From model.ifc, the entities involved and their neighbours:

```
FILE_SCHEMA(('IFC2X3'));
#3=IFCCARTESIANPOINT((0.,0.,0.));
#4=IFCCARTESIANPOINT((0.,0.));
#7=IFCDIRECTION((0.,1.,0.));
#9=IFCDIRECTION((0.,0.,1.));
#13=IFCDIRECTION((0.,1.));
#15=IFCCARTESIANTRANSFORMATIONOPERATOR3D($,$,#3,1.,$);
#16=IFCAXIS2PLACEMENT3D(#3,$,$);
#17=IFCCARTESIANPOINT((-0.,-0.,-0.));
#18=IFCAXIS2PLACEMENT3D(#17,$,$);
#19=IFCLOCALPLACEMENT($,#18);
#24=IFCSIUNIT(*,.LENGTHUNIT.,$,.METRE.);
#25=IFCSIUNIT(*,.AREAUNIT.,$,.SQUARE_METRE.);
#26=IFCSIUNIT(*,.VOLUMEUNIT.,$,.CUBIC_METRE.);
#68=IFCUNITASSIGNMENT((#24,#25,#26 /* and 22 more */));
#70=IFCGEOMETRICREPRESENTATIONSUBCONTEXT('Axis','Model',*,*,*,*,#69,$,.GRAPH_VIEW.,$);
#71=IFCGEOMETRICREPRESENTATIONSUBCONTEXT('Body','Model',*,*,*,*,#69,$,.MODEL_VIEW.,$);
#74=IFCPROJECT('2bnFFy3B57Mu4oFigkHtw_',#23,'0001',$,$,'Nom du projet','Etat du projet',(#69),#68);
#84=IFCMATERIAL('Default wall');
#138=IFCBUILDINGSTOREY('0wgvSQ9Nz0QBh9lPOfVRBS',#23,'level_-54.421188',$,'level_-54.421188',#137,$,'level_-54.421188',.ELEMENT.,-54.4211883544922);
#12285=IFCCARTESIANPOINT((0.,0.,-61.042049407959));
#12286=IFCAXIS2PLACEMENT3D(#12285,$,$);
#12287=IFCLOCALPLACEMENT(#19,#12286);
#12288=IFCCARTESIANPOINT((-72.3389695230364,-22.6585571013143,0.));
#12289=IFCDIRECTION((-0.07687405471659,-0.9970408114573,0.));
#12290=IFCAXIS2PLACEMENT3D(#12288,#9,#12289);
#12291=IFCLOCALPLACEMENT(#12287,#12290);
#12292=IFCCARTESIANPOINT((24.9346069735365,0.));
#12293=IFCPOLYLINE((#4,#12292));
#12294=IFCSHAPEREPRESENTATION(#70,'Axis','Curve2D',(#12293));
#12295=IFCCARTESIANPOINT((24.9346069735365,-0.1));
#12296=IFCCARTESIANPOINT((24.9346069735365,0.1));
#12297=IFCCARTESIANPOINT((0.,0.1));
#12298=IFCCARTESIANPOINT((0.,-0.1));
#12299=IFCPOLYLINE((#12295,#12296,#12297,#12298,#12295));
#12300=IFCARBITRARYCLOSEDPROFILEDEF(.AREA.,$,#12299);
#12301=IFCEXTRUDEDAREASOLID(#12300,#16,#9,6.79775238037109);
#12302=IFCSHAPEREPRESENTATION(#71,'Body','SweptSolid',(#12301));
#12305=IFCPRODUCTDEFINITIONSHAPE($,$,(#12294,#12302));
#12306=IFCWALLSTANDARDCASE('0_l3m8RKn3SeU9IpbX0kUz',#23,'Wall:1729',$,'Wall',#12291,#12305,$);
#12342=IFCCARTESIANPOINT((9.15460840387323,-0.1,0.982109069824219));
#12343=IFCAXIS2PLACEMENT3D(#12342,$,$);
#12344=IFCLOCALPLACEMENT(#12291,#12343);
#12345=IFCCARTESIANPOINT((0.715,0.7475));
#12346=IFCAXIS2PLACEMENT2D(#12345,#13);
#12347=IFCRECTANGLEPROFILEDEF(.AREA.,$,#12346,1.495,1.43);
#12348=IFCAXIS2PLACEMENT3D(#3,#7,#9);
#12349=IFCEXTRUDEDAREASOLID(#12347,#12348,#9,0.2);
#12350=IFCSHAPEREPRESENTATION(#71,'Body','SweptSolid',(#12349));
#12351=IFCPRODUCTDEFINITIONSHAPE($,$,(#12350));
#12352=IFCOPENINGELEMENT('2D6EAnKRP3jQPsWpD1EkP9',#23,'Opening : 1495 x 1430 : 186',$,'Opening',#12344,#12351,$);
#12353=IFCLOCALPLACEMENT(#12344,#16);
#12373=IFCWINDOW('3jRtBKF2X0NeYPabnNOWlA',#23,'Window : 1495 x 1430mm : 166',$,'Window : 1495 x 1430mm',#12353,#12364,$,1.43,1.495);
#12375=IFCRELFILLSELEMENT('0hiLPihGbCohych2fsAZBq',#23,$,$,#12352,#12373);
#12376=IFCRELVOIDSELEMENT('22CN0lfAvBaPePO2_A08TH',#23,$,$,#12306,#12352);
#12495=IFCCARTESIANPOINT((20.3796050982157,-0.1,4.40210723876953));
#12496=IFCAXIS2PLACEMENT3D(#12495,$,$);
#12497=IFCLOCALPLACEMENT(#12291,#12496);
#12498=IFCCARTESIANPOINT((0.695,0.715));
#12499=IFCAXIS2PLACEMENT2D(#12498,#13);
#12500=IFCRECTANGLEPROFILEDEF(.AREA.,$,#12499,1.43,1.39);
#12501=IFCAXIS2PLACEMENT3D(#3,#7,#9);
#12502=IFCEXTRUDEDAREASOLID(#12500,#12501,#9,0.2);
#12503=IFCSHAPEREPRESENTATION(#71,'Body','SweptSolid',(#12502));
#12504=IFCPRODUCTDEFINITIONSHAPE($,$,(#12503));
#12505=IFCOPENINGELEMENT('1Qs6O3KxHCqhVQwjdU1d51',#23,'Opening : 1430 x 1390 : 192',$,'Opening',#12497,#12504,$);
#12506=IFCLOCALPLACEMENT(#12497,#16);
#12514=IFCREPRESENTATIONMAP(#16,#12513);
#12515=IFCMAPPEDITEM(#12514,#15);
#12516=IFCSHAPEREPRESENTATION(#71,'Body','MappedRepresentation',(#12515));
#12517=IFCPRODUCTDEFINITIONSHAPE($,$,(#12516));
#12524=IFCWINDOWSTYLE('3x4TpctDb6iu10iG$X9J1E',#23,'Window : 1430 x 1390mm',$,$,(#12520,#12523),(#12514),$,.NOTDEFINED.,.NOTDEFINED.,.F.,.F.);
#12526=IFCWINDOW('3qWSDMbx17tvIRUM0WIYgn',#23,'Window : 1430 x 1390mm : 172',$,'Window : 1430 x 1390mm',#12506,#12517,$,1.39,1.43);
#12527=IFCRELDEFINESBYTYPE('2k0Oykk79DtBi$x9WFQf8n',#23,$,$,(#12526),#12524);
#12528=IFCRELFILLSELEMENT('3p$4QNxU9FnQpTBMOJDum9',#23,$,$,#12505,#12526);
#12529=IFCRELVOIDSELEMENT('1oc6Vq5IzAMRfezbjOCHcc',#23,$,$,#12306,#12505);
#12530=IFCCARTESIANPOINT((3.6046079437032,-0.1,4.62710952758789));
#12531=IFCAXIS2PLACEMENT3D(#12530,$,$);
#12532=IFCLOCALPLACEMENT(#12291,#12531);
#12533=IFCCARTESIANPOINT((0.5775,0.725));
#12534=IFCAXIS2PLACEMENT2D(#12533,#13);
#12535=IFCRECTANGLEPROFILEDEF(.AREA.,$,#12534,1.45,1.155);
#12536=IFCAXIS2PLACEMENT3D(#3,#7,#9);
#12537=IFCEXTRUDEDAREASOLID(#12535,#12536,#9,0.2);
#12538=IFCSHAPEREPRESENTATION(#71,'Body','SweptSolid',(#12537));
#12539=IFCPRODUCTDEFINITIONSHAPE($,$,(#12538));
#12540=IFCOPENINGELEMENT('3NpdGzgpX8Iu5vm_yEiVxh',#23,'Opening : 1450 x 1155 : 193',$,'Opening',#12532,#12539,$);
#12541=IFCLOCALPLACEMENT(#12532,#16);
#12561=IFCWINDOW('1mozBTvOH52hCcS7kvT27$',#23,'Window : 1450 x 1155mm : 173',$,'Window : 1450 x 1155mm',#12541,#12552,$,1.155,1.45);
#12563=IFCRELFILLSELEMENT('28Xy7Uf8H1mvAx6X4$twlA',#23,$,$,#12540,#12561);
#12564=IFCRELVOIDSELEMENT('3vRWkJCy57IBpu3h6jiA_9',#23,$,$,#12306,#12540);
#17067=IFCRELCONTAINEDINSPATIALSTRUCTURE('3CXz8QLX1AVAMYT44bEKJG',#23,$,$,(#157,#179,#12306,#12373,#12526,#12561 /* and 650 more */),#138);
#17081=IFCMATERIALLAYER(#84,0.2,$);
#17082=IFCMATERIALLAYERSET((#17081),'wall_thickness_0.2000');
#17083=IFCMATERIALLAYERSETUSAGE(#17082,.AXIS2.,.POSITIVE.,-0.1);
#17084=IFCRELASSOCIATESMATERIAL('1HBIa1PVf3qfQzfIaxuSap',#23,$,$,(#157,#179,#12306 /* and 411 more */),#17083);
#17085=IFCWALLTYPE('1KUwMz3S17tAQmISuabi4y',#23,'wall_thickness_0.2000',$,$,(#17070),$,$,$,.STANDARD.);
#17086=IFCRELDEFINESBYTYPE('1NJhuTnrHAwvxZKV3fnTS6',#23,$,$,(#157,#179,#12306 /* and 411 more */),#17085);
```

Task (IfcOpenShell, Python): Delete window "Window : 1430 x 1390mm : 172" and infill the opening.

```python
import ifcopenshell
import ifcopenshell.api.feature
import ifcopenshell.api.root
import ifcopenshell.geom
import ifcopenshell.util.shape

model = ifcopenshell.open("model.ifc")
settings = ifcopenshell.geom.settings()


def volume(element):
    """Net volume in cubic metres, openings subtracted."""
    shape = ifcopenshell.geom.create_shape(settings, element)
    return ifcopenshell.util.shape.get_volume(shape.geometry)


window = model.by_guid("3qWSDMbx17tvIRUM0WIYgn")
opening = window.FillsVoids[0].RelatingOpeningElement
wall = opening.VoidsElements[0].RelatingBuildingElement
before = volume(wall)

ifcopenshell.api.root.remove_product(model, product=window)
ifcopenshell.api.feature.remove_feature(model, feature=opening)

after = volume(wall)

print(f"wall volume {before:.3f} -> {after:.3f} m3")

model.write("model_updated.ifc")
```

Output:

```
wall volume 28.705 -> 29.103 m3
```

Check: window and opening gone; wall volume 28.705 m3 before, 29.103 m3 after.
